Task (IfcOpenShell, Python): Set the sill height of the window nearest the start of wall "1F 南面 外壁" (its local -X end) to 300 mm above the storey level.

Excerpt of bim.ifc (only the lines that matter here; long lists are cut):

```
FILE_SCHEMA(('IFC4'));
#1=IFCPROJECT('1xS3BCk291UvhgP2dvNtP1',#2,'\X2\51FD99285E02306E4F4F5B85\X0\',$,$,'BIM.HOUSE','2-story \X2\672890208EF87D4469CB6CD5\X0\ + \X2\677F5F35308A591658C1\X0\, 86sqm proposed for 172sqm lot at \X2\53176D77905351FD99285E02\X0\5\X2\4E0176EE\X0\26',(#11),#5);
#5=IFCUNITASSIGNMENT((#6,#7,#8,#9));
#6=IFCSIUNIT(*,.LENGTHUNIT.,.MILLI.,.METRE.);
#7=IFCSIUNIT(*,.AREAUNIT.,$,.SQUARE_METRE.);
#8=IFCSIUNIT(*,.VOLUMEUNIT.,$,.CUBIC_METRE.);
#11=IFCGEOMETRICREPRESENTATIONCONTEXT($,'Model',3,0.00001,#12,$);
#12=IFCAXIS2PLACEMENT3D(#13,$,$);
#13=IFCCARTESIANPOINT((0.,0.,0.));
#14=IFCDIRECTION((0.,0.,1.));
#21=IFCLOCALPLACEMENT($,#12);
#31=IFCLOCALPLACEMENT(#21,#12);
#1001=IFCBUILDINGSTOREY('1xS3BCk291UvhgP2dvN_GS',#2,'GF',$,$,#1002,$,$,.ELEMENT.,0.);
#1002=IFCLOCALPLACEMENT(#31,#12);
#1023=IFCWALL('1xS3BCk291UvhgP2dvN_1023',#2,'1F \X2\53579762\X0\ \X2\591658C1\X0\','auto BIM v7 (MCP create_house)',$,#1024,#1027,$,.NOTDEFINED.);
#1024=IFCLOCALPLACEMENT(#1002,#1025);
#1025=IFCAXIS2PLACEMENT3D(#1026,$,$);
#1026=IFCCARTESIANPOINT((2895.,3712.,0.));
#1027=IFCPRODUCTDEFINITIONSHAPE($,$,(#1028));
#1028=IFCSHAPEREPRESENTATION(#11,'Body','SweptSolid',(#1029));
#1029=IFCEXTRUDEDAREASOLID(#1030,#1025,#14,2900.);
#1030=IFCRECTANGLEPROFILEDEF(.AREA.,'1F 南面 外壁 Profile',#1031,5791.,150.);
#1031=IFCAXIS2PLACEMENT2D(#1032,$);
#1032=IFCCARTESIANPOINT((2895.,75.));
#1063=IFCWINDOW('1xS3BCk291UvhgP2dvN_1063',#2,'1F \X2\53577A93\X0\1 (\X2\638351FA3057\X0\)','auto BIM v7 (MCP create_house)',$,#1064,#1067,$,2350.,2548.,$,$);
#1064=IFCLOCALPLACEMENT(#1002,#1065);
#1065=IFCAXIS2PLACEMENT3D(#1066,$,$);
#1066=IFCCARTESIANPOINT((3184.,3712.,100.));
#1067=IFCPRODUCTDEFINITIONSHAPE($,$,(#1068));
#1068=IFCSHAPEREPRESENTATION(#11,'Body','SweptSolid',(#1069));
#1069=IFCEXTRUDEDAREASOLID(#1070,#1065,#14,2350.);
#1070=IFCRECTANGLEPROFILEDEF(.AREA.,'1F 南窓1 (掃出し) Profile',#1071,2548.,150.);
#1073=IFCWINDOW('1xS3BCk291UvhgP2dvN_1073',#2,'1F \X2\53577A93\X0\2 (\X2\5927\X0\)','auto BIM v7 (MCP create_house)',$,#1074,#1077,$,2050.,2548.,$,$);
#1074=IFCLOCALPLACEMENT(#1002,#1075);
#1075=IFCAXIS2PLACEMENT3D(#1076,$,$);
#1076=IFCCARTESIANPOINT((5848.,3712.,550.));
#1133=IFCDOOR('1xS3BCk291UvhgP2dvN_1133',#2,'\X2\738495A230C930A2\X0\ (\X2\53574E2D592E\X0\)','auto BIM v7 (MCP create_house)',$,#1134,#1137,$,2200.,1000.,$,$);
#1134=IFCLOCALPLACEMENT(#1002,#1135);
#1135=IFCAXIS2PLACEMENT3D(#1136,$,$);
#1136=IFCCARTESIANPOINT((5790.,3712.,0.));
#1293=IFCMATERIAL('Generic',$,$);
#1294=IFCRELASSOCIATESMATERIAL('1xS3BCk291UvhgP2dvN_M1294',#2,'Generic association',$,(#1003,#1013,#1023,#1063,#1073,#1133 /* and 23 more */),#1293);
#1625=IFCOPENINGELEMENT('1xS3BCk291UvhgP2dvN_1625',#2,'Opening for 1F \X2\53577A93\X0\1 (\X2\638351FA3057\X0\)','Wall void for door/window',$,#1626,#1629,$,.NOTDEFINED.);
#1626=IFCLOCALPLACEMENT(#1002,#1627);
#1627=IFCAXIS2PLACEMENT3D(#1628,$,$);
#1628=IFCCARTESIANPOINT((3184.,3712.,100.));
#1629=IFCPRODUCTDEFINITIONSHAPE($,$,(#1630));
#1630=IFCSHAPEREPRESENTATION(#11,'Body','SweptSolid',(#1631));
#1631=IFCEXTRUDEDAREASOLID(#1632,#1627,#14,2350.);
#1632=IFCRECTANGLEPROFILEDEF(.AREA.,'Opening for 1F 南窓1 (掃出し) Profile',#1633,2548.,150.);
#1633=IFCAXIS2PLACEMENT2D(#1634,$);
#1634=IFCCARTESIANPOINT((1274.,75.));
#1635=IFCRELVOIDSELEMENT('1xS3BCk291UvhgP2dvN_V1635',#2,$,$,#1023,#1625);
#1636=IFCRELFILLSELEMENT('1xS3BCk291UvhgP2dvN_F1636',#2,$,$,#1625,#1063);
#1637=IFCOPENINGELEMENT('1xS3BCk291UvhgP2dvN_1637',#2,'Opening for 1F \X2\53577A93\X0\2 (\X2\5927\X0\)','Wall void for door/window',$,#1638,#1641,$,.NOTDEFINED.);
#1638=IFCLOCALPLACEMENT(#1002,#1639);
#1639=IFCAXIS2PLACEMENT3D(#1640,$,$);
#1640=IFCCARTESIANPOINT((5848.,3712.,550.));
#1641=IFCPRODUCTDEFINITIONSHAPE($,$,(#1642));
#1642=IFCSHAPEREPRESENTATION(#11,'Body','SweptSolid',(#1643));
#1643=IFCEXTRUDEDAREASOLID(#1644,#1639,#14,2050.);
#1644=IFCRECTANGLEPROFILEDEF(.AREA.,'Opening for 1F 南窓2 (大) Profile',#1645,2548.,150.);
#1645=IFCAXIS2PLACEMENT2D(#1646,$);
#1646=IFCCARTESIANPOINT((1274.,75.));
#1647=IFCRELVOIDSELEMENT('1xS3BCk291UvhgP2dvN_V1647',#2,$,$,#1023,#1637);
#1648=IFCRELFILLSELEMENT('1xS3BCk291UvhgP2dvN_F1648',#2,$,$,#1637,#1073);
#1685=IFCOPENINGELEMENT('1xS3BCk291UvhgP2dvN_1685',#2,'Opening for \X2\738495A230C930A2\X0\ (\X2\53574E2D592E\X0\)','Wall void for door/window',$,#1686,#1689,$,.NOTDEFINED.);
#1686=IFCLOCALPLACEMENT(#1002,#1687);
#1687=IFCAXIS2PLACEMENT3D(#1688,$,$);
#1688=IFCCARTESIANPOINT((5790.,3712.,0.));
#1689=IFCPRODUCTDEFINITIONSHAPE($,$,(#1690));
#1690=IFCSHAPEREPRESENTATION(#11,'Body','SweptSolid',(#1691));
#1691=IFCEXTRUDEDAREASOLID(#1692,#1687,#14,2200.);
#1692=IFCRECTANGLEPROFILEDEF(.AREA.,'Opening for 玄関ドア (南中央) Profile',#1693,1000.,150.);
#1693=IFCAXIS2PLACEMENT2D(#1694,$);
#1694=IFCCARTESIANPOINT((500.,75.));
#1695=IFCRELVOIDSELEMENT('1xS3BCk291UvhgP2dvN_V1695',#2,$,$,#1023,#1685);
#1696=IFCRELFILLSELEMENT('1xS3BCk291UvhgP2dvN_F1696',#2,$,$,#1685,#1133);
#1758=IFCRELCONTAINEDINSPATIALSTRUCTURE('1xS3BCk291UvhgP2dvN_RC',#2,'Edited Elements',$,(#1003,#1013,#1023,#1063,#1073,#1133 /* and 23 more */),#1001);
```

```python
import numpy as np
import ifcopenshell
import ifcopenshell.api.geometry
import ifcopenshell.geom
import ifcopenshell.util.element
import ifcopenshell.util.placement
import ifcopenshell.util.shape
import ifcopenshell.util.unit

model = ifcopenshell.open("bim.ifc")
unit_scale = ifcopenshell.util.unit.calculate_unit_scale(model)

window = model.by_guid("1xS3BCk291UvhgP2dvN_1063")
opening = window.FillsVoids[0].RelatingOpeningElement
storey = ifcopenshell.util.element.get_container(window, ifc_class="IfcBuildingStorey")
level = ifcopenshell.util.placement.get_local_placement(storey.ObjectPlacement)[2, 3]

# The opening's origin need not be at the sill, so measure its lowest point.
shape = ifcopenshell.geom.create_shape(ifcopenshell.geom.settings(), opening)
bottom = ifcopenshell.util.shape.get_shape_bottom_elevation(shape, shape.geometry) / unit_scale
dz = level + 0.3 / unit_scale - bottom

shift = np.array([0.0, 0.0, dz])
# The window is not placed relative to its opening, so move both.
for product in (opening, window):
    matrix = ifcopenshell.util.placement.get_local_placement(product.ObjectPlacement)
    matrix[:3, 3] += shift
    ifcopenshell.api.geometry.edit_object_placement(model, product=product, matrix=matrix, is_si=False)

print(f"moved by {dz * unit_scale:+.3f} m")

model.write("bim_v2.ifc")
```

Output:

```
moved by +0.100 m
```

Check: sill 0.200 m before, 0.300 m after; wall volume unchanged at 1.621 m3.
